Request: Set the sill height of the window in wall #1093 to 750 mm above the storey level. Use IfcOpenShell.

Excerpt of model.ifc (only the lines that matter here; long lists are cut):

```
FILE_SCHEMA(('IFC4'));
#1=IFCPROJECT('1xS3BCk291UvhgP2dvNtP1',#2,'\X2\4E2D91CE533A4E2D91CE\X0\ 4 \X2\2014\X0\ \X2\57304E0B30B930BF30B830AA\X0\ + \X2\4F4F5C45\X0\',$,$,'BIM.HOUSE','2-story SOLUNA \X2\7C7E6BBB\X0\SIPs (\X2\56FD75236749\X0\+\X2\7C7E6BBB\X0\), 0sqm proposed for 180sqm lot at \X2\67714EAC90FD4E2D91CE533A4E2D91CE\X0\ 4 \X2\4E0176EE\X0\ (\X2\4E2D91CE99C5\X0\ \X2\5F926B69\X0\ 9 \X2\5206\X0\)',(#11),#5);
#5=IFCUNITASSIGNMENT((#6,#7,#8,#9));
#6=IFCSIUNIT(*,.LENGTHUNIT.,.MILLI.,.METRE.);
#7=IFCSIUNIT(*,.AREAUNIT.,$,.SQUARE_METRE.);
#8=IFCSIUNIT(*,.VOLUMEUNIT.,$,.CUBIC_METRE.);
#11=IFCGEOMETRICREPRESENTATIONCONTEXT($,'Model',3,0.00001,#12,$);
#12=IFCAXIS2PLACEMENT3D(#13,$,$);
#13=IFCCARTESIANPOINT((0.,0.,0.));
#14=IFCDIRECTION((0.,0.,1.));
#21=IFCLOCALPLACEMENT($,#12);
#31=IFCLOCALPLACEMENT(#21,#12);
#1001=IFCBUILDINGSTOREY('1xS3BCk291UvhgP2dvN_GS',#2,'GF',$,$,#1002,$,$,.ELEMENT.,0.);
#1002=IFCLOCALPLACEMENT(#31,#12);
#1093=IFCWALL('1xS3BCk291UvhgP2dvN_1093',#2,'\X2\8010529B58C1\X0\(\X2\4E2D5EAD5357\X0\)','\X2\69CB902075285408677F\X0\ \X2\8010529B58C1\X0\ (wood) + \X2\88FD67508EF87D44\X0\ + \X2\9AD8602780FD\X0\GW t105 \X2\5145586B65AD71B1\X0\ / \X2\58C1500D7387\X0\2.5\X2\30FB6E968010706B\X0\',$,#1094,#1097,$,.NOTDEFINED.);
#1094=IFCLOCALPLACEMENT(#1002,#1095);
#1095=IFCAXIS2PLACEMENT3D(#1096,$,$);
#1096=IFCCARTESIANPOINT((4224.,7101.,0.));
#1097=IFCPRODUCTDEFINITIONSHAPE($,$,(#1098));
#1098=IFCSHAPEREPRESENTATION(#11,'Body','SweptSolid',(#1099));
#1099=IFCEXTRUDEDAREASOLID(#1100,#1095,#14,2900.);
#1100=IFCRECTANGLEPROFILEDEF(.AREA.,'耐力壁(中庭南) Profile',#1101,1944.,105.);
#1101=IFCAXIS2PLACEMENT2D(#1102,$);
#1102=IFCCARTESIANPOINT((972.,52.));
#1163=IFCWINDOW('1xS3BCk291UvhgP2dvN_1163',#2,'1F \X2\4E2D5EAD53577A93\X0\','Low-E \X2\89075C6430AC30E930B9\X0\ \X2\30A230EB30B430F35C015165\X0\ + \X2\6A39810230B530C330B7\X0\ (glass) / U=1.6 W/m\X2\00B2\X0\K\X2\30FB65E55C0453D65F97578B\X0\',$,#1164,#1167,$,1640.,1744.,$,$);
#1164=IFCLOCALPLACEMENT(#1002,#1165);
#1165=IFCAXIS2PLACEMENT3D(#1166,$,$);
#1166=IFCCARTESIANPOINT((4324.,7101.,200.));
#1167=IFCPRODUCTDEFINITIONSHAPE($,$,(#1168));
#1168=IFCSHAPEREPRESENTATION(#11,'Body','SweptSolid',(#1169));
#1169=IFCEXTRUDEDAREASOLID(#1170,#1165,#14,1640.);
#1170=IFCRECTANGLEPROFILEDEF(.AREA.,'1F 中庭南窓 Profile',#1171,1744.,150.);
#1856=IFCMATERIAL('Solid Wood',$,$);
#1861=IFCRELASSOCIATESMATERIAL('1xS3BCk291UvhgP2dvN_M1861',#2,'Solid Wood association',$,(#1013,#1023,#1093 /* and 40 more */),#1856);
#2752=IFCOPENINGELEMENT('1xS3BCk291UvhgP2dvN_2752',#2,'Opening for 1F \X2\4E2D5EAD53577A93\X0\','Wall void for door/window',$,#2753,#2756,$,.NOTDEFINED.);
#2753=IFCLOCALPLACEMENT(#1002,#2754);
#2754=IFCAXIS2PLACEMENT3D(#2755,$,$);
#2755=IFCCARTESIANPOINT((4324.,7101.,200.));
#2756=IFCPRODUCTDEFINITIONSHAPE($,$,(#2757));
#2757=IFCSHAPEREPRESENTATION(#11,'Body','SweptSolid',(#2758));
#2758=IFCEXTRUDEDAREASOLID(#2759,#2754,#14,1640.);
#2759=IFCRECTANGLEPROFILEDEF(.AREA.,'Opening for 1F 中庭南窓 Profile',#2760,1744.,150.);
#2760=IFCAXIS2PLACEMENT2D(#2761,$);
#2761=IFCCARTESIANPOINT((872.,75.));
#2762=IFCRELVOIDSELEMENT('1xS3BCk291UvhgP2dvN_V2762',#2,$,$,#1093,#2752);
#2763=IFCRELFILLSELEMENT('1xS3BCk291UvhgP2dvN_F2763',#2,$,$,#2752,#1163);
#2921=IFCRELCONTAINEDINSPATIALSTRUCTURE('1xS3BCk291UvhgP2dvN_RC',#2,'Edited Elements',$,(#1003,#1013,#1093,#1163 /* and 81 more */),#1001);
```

```python
import numpy as np
import ifcopenshell
import ifcopenshell.api.geometry
import ifcopenshell.geom
import ifcopenshell.util.element
import ifcopenshell.util.placement
import ifcopenshell.util.shape
import ifcopenshell.util.unit

model = ifcopenshell.open("model.ifc")
unit_scale = ifcopenshell.util.unit.calculate_unit_scale(model)

window = model.by_guid("1xS3BCk291UvhgP2dvN_1163")
opening = window.FillsVoids[0].RelatingOpeningElement
storey = ifcopenshell.util.element.get_container(window, ifc_class="IfcBuildingStorey")
level = ifcopenshell.util.placement.get_local_placement(storey.ObjectPlacement)[2, 3]

# The opening's origin need not be at the sill, so measure its lowest point.
shape = ifcopenshell.geom.create_shape(ifcopenshell.geom.settings(), opening)
bottom = ifcopenshell.util.shape.get_shape_bottom_elevation(shape, shape.geometry) / unit_scale
dz = level + 0.75 / unit_scale - bottom

shift = np.array([0.0, 0.0, dz])
# The window is not placed relative to its opening, so move both.
for product in (opening, window):
    matrix = ifcopenshell.util.placement.get_local_placement(product.ObjectPlacement)
    matrix[:3, 3] += shift
    ifcopenshell.api.geometry.edit_object_placement(model, product=product, matrix=matrix, is_si=False)

print(f"moved by {dz * unit_scale:+.3f} m")

model.write("model_edited.ifc")
```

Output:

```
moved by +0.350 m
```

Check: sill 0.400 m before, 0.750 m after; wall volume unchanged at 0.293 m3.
